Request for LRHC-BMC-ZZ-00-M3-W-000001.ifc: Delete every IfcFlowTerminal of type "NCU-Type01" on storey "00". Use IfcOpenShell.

First a look at what the model holds.

```python
import ifcopenshell
import ifcopenshell.util.element

model = ifcopenshell.open("LRHC-BMC-ZZ-00-M3-W-000001.ifc")
print(model.schema)
storey = next(s for s in model.by_type("IfcBuildingStorey") if s.Name == "00")
terminals = [e for e in ifcopenshell.util.element.get_decomposition(storey) if e.is_a("IfcFlowTerminal")]
seen = {}
for e in terminals:
    element_type = ifcopenshell.util.element.get_type(e)
    name = element_type.Name if element_type not in (None, e) else None
    seen[name] = seen.get(name, 0) + 1
for name, count in sorted(seen.items(), key=str):
    print(count, "x", name)
```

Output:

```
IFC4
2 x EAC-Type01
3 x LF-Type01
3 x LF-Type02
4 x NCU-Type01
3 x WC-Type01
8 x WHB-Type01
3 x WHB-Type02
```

```python
import ifcopenshell
import ifcopenshell.api.root
import ifcopenshell.util.element

model = ifcopenshell.open("LRHC-BMC-ZZ-00-M3-W-000001.ifc")

storey = next(s for s in model.by_type("IfcBuildingStorey") if s.Name == "00")
terminals = [e for e in ifcopenshell.util.element.get_decomposition(storey) if e.is_a("IfcFlowTerminal")]
targets = [e for e in terminals if (t := ifcopenshell.util.element.get_type(e)) not in (None, e) and t.Name == "NCU-Type01"]

for e in targets:
    ifcopenshell.api.root.remove_product(model, product=e)
print(len(targets), "removed")

model.write("LRHC-BMC-ZZ-00-M3-W-000001_rev.ifc")
```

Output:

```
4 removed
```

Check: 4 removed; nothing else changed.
